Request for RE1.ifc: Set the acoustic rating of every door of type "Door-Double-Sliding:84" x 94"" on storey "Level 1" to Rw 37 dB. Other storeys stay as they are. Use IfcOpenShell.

First a look at what the model holds.

```python
import ifcopenshell
import ifcopenshell.util.element

model = ifcopenshell.open("RE1.ifc")
print(model.schema)
storey = next(s for s in model.by_type("IfcBuildingStorey") if s.Name == "Level 1")
doors = [e for e in ifcopenshell.util.element.get_decomposition(storey) if e.is_a("IfcDoor")]
seen = {}
for e in doors:
    element_type = ifcopenshell.util.element.get_type(e)
    key = (element_type.Name if element_type != e and element_type else None, ifcopenshell.util.element.get_pset(e, "Pset_DoorCommon", "AcousticRating"))
    seen[key] = seen.get(key, 0) + 1
for (name, value), count in sorted(seen.items(), key=str):
    print(count, "x", name, "|", value)
```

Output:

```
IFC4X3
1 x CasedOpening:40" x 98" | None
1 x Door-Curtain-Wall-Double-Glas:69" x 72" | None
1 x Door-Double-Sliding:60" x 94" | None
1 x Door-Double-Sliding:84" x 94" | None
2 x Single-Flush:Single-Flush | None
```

```python
import ifcopenshell
import ifcopenshell.api.pset
import ifcopenshell.util.element

model = ifcopenshell.open("RE1.ifc")

storey = next(s for s in model.by_type("IfcBuildingStorey") if s.Name == "Level 1")
doors = [e for e in ifcopenshell.util.element.get_decomposition(storey) if e.is_a("IfcDoor")]

count = 0
for e in doors:
    element_type = ifcopenshell.util.element.get_type(e)
    if element_type in (None, e) or element_type.Name != 'Door-Double-Sliding:84" x 94"':
        continue
    # add_pset returns the element's existing set when there is one.
    pset = ifcopenshell.api.pset.add_pset(model, product=e, name="Pset_DoorCommon")
    ifcopenshell.api.pset.edit_pset(model, pset=pset, properties={"AcousticRating": "Rw 37 dB"})
    count += 1

print(count, "doors updated")

model.write("RE1-out.ifc")
```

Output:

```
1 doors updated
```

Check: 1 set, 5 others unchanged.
